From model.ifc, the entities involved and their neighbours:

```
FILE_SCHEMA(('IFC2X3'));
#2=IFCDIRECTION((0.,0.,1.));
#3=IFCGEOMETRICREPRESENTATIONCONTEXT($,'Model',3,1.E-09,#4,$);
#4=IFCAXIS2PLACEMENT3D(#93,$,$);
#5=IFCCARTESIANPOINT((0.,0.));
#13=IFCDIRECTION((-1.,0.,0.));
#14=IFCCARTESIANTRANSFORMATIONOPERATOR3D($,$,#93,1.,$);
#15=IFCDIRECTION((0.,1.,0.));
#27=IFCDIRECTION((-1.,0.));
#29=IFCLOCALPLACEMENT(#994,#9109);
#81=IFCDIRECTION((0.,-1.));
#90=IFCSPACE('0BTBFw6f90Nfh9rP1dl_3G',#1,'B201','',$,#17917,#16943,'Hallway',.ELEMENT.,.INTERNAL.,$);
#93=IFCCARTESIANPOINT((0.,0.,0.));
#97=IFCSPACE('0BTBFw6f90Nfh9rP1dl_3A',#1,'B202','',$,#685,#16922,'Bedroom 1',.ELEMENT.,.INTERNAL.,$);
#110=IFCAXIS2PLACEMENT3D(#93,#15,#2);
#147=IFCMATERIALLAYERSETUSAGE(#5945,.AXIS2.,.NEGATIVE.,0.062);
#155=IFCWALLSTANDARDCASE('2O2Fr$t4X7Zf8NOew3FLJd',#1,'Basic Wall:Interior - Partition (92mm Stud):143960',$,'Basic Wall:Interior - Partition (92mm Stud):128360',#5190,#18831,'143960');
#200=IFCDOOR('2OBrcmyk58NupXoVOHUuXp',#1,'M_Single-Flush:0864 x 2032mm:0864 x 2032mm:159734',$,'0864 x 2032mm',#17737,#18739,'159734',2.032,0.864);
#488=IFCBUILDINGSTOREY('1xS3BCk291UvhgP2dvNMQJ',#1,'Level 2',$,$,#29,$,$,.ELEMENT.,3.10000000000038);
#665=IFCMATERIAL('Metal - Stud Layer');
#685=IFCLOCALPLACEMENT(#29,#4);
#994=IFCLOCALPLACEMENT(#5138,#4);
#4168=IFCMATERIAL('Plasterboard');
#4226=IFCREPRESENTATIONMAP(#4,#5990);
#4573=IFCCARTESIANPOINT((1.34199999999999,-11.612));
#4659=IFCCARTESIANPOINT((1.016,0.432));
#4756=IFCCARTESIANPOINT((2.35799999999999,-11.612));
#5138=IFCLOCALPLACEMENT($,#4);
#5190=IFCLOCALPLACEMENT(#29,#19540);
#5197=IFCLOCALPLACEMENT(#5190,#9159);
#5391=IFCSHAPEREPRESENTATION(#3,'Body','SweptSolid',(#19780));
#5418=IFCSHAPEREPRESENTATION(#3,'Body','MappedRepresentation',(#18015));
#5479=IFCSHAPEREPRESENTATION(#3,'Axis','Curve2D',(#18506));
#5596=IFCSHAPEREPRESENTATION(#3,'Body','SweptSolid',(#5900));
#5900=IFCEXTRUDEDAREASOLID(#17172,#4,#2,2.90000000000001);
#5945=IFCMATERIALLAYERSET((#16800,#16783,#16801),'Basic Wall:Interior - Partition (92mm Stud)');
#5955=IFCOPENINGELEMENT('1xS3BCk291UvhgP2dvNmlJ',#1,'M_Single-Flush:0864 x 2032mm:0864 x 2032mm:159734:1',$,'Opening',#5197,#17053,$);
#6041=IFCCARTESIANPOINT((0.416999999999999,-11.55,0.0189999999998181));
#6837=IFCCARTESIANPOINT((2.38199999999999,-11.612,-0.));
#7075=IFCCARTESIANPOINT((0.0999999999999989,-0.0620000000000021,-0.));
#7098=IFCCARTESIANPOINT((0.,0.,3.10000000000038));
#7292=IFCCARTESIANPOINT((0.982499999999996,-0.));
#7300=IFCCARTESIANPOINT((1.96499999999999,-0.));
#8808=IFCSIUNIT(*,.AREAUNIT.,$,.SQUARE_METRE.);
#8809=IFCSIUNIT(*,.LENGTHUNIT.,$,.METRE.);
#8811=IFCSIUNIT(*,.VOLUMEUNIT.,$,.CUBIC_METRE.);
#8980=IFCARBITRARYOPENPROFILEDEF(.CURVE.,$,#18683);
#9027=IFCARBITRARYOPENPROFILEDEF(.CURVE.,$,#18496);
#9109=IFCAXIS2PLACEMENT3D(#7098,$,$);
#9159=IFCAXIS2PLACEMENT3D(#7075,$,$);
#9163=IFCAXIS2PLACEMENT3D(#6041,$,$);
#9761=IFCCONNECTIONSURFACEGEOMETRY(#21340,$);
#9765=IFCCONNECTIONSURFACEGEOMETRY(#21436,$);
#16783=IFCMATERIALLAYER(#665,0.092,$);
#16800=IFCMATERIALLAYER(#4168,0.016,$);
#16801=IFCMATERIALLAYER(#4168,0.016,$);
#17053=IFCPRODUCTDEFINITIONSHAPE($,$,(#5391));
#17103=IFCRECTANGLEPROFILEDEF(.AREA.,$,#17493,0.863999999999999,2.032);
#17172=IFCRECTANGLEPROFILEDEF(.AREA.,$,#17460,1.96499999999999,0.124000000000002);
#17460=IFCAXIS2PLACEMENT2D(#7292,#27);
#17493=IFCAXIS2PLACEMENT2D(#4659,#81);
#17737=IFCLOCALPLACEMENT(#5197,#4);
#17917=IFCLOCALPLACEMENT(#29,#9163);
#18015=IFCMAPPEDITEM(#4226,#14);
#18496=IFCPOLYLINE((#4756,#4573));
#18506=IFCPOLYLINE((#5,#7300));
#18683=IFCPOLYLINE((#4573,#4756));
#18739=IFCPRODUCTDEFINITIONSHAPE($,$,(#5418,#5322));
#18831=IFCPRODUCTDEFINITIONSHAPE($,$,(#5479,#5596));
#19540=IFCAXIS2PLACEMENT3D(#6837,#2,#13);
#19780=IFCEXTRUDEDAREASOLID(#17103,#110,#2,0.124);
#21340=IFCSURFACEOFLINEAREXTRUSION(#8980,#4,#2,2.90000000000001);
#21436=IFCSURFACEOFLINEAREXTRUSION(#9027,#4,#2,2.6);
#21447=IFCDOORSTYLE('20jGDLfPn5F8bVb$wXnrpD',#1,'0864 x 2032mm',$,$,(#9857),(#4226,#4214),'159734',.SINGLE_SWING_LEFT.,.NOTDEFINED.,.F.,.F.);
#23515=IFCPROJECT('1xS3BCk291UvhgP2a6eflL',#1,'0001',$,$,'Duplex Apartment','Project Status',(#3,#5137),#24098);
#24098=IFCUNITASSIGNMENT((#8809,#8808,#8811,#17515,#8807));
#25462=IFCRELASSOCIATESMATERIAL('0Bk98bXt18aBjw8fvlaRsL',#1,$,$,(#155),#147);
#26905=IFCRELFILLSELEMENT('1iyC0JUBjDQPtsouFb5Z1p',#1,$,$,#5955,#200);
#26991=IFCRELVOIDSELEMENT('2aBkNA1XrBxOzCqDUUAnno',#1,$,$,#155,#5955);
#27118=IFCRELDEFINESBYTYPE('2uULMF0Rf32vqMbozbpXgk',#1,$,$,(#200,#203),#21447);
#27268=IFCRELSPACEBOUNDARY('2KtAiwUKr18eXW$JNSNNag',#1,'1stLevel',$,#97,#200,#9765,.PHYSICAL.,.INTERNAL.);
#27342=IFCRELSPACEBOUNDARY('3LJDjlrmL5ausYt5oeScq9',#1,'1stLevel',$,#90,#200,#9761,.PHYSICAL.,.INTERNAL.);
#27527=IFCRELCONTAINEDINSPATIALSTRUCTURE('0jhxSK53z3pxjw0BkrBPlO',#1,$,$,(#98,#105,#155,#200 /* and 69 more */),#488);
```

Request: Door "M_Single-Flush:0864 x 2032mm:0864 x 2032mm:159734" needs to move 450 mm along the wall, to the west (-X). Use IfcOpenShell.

```python
import numpy as np
import ifcopenshell
import ifcopenshell.api.geometry
import ifcopenshell.util.placement
import ifcopenshell.util.unit

model = ifcopenshell.open("model.ifc")
unit_scale = ifcopenshell.util.unit.calculate_unit_scale(model)

door = model.by_guid("2OBrcmyk58NupXoVOHUuXp")
opening = door.FillsVoids[0].RelatingOpeningElement
wall = opening.VoidsElements[0].RelatingBuildingElement

wall_matrix = ifcopenshell.util.placement.get_local_placement(wall.ObjectPlacement)
shift = wall_matrix[:3, 0] * 0.45 / unit_scale
before = ifcopenshell.util.placement.get_local_placement(door.ObjectPlacement)[:3, 3].copy()

# The door is placed relative to its opening, so it follows when the opening moves.
matrix = ifcopenshell.util.placement.get_local_placement(opening.ObjectPlacement)
matrix[:3, 3] += shift
ifcopenshell.api.geometry.edit_object_placement(
    model, product=opening, matrix=matrix, is_si=False, should_transform_children=True
)

# Space boundary surfaces are stored in each space's coordinates; move them too.
for rel in door.ProvidesBoundaries:
    if not rel.ConnectionGeometry:
        continue
    surface = rel.ConnectionGeometry.SurfaceOnRelatingElement
    space_matrix = ifcopenshell.util.placement.get_local_placement(rel.RelatingSpace.ObjectPlacement)
    point = np.array(surface.Position.Location.Coordinates) + space_matrix[:3, :3].T @ shift
    surface.Position = model.createIfcAxis2Placement3D(
        model.createIfcCartesianPoint(point.tolist()), surface.Position.Axis, surface.Position.RefDirection
    )

after = ifcopenshell.util.placement.get_local_placement(door.ObjectPlacement)[:3, 3]
print("door moved by", (after - before).round(3) + 0.0)

model.write("model_v2.ifc")
```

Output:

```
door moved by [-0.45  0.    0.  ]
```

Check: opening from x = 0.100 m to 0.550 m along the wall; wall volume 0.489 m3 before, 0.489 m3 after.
